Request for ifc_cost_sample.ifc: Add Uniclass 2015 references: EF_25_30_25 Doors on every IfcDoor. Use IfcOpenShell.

First a look at what the model holds.

```python
import ifcopenshell

model = ifcopenshell.open("ifc_cost_sample.ifc")
print(model.schema)
print("classifications:", [c.Name for c in model.by_type("IfcClassification")])
for ifc_class in ("IfcDoor", "IfcRoof", "IfcStair", "IfcWall", "IfcWindow"):
    print(ifc_class, len(model.by_type(ifc_class)))
```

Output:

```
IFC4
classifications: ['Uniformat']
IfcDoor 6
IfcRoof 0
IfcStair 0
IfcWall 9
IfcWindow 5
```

```python
import ifcopenshell
import ifcopenshell.api.classification

model = ifcopenshell.open("ifc_cost_sample.ifc")

system = ifcopenshell.api.classification.add_classification(model, classification="Uniclass 2015")

codes = {
    "IfcDoor": ("EF_25_30_25", "Doors"),
}
for ifc_class, (code, name) in codes.items():
    products = model.by_type(ifc_class)
    ifcopenshell.api.classification.add_reference(
        model, products=products, classification=system, identification=code, name=name
    )
    print(code, len(products))

model.write("ifc_cost_sample_edited.ifc")
```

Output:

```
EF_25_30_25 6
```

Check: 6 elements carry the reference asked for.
